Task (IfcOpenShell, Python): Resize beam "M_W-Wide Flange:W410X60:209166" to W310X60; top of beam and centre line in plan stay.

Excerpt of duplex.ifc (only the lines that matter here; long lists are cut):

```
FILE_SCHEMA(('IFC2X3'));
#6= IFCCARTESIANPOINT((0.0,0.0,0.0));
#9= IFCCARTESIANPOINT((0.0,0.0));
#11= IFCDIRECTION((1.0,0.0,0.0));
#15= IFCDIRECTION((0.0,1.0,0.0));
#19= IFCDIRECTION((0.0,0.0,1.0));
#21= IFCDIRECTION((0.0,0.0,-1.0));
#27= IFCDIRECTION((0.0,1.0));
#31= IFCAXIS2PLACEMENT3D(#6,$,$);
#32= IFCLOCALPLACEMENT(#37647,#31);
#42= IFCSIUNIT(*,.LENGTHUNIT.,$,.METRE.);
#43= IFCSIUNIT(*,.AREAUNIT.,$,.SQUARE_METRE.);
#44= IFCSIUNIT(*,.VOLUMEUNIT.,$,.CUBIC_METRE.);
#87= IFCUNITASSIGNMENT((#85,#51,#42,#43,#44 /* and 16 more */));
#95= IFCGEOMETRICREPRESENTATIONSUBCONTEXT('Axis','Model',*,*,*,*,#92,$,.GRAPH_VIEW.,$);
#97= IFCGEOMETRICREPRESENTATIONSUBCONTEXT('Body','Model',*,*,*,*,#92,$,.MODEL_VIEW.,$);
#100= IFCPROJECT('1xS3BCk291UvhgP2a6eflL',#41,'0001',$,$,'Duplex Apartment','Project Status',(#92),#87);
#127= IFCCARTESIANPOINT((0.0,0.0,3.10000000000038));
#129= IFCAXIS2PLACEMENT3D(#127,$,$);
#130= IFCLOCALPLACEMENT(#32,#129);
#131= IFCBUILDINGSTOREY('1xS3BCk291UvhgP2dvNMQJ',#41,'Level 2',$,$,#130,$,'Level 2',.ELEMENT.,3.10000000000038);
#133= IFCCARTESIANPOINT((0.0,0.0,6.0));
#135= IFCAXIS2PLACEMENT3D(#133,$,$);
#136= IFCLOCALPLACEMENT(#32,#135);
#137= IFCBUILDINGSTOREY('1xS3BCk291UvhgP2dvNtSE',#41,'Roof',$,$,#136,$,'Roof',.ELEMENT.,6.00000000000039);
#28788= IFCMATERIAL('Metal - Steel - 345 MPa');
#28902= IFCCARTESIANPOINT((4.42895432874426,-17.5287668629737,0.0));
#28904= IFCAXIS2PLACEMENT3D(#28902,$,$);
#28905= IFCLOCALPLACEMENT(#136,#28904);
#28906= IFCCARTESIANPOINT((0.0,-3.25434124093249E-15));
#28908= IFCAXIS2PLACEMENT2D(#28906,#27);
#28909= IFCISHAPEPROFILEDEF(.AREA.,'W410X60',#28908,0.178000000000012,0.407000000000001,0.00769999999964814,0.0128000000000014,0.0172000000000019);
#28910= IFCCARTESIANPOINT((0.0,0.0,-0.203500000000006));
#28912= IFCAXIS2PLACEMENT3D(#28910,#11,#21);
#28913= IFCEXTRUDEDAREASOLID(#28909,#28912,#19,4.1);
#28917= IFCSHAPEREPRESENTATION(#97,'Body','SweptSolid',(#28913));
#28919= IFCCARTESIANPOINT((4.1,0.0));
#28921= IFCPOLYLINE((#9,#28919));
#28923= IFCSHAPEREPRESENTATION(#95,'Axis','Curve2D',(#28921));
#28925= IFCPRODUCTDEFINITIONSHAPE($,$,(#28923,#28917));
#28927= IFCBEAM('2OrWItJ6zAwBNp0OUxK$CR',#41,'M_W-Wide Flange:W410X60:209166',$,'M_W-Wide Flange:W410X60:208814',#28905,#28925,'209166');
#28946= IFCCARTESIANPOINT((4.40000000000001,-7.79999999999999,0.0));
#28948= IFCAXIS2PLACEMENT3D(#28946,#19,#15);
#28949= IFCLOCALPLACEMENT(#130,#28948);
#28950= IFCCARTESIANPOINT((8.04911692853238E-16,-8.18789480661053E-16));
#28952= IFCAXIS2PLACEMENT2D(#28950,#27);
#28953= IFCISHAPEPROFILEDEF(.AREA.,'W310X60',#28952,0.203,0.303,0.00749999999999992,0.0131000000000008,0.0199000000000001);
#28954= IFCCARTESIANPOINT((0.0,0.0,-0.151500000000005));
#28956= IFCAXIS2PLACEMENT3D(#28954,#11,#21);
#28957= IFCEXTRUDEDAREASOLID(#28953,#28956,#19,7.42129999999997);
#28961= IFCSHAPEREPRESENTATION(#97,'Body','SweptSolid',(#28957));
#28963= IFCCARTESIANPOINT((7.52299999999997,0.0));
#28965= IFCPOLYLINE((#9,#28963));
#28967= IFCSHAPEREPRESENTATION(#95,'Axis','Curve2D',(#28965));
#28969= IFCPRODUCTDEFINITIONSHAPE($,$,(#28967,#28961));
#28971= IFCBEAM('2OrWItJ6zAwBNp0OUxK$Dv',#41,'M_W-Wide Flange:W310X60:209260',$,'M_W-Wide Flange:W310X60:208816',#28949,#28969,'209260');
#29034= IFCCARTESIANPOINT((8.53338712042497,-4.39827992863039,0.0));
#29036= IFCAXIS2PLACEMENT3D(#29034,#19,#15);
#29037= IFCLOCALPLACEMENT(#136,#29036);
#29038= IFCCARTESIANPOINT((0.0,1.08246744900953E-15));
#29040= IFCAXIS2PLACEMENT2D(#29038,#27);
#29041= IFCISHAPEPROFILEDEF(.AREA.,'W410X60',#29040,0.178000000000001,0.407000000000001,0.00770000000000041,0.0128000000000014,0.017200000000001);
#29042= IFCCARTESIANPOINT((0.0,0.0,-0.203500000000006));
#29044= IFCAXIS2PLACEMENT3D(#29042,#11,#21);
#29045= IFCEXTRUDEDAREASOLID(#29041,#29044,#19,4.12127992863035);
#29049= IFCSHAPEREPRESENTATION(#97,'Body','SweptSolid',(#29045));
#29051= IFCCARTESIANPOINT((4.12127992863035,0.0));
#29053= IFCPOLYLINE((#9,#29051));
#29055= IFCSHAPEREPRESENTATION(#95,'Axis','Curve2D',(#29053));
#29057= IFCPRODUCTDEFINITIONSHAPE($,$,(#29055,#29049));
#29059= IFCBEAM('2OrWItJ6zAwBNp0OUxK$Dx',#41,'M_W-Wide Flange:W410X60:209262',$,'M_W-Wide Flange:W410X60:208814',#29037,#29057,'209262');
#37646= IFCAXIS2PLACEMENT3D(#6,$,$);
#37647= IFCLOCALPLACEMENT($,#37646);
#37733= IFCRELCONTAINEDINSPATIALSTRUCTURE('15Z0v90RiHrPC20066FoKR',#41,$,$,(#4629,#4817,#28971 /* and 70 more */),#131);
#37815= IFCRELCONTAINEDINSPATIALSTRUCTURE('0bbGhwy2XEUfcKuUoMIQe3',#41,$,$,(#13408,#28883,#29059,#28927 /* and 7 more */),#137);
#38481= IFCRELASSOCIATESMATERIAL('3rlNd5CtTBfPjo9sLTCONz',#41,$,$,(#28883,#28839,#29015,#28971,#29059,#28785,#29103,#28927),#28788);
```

```python
import ifcopenshell
import ifcopenshell.util.element
import ifcopenshell.util.representation

model = ifcopenshell.open("duplex.ifc")

member = model.by_guid("2OrWItJ6zAwBNp0OUxK$CR")
source = next(p for p in model.by_type("IfcIShapeProfileDef") if p.ProfileName == "W310X60")

body = ifcopenshell.util.representation.get_representation(member, "Model", "Body")
solid = body.Items[0]
old_profile = solid.SweptArea

# Copy the section's sizes but keep this member's own profile position.
profile = ifcopenshell.util.element.copy(model, source)
# Profiles are centred, so shift by half the change in depth to hold the top.
shift = (old_profile.OverallDepth - profile.OverallDepth) / 2
x, y = old_profile.Position.Location.Coordinates
up = (-1.0, 0.0)  # upwards, in the solid's own plane
location = model.createIfcCartesianPoint((x + up[0] * shift, y + up[1] * shift))
profile.Position = model.createIfcAxis2Placement2D(location, old_profile.Position.RefDirection)
solid.SweptArea = profile
if not model.get_total_inverses(old_profile):
    ifcopenshell.util.element.remove_deep2(model, old_profile)
member.Name = member.Name.replace("W410X60", "W310X60")
member.ObjectType = member.ObjectType.replace("W410X60", "W310X60")

print(solid.SweptArea)

model.write("duplex_v2.ifc")
```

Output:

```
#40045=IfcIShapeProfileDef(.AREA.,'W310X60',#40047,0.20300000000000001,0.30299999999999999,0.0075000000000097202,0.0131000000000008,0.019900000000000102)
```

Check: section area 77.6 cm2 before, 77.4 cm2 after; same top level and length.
